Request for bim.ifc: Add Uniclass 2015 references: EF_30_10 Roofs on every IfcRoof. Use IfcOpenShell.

First a look at what the model holds.

```python
import ifcopenshell

model = ifcopenshell.open("bim.ifc")
print(model.schema)
print("classifications:", [c.Name for c in model.by_type("IfcClassification")])
for ifc_class in ("IfcDoor", "IfcRoof", "IfcStair", "IfcWall", "IfcWindow"):
    print(ifc_class, len(model.by_type(ifc_class)))
```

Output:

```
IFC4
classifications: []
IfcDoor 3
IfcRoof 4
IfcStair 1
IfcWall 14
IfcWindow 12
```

```python
import ifcopenshell
import ifcopenshell.api.classification

model = ifcopenshell.open("bim.ifc")

system = ifcopenshell.api.classification.add_classification(model, classification="Uniclass 2015")

codes = {
    "IfcRoof": ("EF_30_10", "Roofs"),
}
for ifc_class, (code, name) in codes.items():
    products = model.by_type(ifc_class)
    ifcopenshell.api.classification.add_reference(
        model, products=products, classification=system, identification=code, name=name
    )
    print(code, len(products))

model.write("bim-out.ifc")
```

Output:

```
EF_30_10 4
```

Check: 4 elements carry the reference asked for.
